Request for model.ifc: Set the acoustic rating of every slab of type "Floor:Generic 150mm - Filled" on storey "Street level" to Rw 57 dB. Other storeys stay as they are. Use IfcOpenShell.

First a look at what the model holds.

```python
import ifcopenshell
import ifcopenshell.util.element

model = ifcopenshell.open("model.ifc")
print(model.schema)
storey = next(s for s in model.by_type("IfcBuildingStorey") if s.Name == "Street level")
slabs = [e for e in ifcopenshell.util.element.get_decomposition(storey) if e.is_a("IfcSlab")]
seen = {}
for e in slabs:
    element_type = ifcopenshell.util.element.get_type(e)
    key = (element_type.Name if element_type != e and element_type else None, ifcopenshell.util.element.get_pset(e, "Pset_SlabCommon", "AcousticRating"))
    seen[key] = seen.get(key, 0) + 1
for (name, value), count in sorted(seen.items(), key=str):
    print(count, "x", name, "|", value)
```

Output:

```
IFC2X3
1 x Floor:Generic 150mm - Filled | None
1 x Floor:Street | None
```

```python
import ifcopenshell
import ifcopenshell.api.pset
import ifcopenshell.util.element

model = ifcopenshell.open("model.ifc")

storey = next(s for s in model.by_type("IfcBuildingStorey") if s.Name == "Street level")
slabs = [e for e in ifcopenshell.util.element.get_decomposition(storey) if e.is_a("IfcSlab")]

count = 0
for e in slabs:
    element_type = ifcopenshell.util.element.get_type(e)
    if element_type in (None, e) or element_type.Name != "Floor:Generic 150mm - Filled":
        continue
    # add_pset returns the element's existing set when there is one.
    pset = ifcopenshell.api.pset.add_pset(model, product=e, name="Pset_SlabCommon")
    ifcopenshell.api.pset.edit_pset(model, pset=pset, properties={"AcousticRating": "Rw 57 dB"})
    count += 1

print(count, "slabs updated")

model.write("model_rev.ifc")
```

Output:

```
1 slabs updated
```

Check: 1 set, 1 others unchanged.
